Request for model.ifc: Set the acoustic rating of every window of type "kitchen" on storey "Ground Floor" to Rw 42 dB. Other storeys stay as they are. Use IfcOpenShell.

First a look at what the model holds.

```python
import ifcopenshell
import ifcopenshell.util.element

model = ifcopenshell.open("model.ifc")
print(model.schema)
storey = next(s for s in model.by_type("IfcBuildingStorey") if s.Name == "Ground Floor")
windows = [e for e in ifcopenshell.util.element.get_decomposition(storey) if e.is_a("IfcWindow")]
seen = {}
for e in windows:
    element_type = ifcopenshell.util.element.get_type(e)
    key = (element_type.Name if element_type != e and element_type else None, ifcopenshell.util.element.get_pset(e, "Pset_WindowCommon", "AcousticRating"))
    seen[key] = seen.get(key, 0) + 1
for (name, value), count in sorted(seen.items(), key=str):
    print(count, "x", name, "|", value)
```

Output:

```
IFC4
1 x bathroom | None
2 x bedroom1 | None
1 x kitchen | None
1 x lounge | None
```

```python
import ifcopenshell
import ifcopenshell.api.pset
import ifcopenshell.util.element

model = ifcopenshell.open("model.ifc")

storey = next(s for s in model.by_type("IfcBuildingStorey") if s.Name == "Ground Floor")
windows = [e for e in ifcopenshell.util.element.get_decomposition(storey) if e.is_a("IfcWindow")]

count = 0
for e in windows:
    element_type = ifcopenshell.util.element.get_type(e)
    if element_type in (None, e) or element_type.Name != "kitchen":
        continue
    # add_pset returns the element's existing set when there is one.
    pset = ifcopenshell.api.pset.add_pset(model, product=e, name="Pset_WindowCommon")
    ifcopenshell.api.pset.edit_pset(model, pset=pset, properties={"AcousticRating": "Rw 42 dB"})
    count += 1

print(count, "windows updated")

model.write("model_updated.ifc")
```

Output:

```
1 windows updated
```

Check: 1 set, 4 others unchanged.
